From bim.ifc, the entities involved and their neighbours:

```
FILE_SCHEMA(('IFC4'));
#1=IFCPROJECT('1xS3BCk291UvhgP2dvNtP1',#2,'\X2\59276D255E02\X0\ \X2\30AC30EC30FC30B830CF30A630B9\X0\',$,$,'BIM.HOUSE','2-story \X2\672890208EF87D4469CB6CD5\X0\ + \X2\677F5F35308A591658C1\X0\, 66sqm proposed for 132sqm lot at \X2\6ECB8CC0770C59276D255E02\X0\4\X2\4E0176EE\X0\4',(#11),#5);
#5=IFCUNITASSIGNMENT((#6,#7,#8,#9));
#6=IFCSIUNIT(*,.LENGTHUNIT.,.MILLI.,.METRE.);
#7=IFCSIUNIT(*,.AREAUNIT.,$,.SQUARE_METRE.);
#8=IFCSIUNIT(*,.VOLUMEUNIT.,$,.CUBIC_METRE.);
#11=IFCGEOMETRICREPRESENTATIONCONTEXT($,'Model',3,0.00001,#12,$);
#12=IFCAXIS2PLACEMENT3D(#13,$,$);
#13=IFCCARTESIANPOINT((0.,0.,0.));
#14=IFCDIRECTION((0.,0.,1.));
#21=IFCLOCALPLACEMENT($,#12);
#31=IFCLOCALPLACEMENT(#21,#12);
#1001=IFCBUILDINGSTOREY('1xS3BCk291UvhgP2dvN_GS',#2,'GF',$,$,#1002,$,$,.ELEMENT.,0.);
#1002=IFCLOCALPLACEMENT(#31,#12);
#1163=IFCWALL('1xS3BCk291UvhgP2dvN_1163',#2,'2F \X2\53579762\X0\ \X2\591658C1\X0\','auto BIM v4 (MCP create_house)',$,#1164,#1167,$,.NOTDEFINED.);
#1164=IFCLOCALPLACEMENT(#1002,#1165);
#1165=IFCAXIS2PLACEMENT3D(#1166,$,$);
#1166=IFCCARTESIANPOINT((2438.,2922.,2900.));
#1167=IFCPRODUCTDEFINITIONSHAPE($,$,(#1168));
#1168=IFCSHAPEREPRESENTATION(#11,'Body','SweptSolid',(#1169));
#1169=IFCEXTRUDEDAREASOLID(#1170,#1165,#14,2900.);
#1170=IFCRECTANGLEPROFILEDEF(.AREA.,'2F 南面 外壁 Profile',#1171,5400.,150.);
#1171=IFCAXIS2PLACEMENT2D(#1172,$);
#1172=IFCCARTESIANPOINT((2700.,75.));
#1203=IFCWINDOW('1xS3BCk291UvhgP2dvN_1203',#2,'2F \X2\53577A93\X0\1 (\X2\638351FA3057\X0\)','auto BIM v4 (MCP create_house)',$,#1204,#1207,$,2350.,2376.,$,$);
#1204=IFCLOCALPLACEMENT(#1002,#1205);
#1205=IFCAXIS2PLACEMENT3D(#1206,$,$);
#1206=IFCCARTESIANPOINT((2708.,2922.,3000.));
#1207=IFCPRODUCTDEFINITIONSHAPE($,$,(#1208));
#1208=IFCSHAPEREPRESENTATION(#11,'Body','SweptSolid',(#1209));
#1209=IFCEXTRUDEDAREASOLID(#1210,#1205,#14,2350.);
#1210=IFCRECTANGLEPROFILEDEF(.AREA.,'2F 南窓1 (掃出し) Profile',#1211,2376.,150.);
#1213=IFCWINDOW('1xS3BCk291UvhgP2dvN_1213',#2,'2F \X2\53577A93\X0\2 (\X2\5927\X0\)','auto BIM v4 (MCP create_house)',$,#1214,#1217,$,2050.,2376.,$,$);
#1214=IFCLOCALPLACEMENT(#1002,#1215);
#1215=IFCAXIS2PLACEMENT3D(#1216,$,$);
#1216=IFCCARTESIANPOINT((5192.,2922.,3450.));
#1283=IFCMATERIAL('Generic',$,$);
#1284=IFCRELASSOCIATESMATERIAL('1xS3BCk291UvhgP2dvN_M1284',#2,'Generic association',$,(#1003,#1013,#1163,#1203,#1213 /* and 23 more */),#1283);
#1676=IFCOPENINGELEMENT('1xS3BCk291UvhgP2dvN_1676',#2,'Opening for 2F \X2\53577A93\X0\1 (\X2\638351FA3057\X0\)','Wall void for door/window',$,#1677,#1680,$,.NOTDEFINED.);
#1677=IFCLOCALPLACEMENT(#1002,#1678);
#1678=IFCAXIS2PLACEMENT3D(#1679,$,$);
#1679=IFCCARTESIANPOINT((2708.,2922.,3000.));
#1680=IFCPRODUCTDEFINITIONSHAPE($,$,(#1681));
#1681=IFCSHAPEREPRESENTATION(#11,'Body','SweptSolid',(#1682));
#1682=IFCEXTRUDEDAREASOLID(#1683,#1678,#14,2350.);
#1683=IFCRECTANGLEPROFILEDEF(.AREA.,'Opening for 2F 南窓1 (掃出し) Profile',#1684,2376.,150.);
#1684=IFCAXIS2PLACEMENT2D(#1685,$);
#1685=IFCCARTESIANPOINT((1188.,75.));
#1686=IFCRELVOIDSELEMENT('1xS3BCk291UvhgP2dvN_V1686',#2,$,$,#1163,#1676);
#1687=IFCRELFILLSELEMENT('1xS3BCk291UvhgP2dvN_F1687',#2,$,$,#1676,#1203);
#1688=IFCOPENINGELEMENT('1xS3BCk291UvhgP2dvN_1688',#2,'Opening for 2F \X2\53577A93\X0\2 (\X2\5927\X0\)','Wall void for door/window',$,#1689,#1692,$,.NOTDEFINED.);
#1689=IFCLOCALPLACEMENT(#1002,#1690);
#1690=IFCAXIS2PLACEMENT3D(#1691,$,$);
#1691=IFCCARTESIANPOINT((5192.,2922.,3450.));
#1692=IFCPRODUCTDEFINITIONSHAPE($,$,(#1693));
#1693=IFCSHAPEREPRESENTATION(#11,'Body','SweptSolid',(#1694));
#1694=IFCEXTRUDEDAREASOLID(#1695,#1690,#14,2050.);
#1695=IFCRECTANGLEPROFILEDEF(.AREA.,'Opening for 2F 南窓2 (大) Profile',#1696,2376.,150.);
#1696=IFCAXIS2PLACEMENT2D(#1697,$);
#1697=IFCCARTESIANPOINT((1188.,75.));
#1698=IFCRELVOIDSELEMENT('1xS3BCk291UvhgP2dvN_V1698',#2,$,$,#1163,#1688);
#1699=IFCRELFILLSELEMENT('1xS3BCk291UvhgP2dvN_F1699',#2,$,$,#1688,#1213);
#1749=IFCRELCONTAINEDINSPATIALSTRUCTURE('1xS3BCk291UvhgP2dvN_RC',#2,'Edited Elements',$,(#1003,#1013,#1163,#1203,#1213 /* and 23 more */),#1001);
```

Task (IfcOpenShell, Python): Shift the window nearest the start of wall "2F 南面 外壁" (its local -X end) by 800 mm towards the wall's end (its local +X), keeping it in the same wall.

```python
import ifcopenshell
import ifcopenshell.api.geometry
import ifcopenshell.util.placement
import ifcopenshell.util.unit

model = ifcopenshell.open("bim.ifc")
unit_scale = ifcopenshell.util.unit.calculate_unit_scale(model)

window = model.by_guid("1xS3BCk291UvhgP2dvN_1203")
opening = window.FillsVoids[0].RelatingOpeningElement
wall = opening.VoidsElements[0].RelatingBuildingElement

wall_matrix = ifcopenshell.util.placement.get_local_placement(wall.ObjectPlacement)
shift = wall_matrix[:3, 0] * 0.8 / unit_scale
before = ifcopenshell.util.placement.get_local_placement(window.ObjectPlacement)[:3, 3].copy()

# The window is not placed relative to its opening, so move both.
for product in (opening, window):
    matrix = ifcopenshell.util.placement.get_local_placement(product.ObjectPlacement)
    matrix[:3, 3] += shift
    ifcopenshell.api.geometry.edit_object_placement(model, product=product, matrix=matrix, is_si=False)

after = ifcopenshell.util.placement.get_local_placement(window.ObjectPlacement)[:3, 3]
print("window moved by", (after - before).round(3) + 0.0)

model.write("bim_edited.ifc")
```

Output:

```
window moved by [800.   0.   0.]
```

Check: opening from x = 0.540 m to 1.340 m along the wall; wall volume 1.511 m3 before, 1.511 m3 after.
